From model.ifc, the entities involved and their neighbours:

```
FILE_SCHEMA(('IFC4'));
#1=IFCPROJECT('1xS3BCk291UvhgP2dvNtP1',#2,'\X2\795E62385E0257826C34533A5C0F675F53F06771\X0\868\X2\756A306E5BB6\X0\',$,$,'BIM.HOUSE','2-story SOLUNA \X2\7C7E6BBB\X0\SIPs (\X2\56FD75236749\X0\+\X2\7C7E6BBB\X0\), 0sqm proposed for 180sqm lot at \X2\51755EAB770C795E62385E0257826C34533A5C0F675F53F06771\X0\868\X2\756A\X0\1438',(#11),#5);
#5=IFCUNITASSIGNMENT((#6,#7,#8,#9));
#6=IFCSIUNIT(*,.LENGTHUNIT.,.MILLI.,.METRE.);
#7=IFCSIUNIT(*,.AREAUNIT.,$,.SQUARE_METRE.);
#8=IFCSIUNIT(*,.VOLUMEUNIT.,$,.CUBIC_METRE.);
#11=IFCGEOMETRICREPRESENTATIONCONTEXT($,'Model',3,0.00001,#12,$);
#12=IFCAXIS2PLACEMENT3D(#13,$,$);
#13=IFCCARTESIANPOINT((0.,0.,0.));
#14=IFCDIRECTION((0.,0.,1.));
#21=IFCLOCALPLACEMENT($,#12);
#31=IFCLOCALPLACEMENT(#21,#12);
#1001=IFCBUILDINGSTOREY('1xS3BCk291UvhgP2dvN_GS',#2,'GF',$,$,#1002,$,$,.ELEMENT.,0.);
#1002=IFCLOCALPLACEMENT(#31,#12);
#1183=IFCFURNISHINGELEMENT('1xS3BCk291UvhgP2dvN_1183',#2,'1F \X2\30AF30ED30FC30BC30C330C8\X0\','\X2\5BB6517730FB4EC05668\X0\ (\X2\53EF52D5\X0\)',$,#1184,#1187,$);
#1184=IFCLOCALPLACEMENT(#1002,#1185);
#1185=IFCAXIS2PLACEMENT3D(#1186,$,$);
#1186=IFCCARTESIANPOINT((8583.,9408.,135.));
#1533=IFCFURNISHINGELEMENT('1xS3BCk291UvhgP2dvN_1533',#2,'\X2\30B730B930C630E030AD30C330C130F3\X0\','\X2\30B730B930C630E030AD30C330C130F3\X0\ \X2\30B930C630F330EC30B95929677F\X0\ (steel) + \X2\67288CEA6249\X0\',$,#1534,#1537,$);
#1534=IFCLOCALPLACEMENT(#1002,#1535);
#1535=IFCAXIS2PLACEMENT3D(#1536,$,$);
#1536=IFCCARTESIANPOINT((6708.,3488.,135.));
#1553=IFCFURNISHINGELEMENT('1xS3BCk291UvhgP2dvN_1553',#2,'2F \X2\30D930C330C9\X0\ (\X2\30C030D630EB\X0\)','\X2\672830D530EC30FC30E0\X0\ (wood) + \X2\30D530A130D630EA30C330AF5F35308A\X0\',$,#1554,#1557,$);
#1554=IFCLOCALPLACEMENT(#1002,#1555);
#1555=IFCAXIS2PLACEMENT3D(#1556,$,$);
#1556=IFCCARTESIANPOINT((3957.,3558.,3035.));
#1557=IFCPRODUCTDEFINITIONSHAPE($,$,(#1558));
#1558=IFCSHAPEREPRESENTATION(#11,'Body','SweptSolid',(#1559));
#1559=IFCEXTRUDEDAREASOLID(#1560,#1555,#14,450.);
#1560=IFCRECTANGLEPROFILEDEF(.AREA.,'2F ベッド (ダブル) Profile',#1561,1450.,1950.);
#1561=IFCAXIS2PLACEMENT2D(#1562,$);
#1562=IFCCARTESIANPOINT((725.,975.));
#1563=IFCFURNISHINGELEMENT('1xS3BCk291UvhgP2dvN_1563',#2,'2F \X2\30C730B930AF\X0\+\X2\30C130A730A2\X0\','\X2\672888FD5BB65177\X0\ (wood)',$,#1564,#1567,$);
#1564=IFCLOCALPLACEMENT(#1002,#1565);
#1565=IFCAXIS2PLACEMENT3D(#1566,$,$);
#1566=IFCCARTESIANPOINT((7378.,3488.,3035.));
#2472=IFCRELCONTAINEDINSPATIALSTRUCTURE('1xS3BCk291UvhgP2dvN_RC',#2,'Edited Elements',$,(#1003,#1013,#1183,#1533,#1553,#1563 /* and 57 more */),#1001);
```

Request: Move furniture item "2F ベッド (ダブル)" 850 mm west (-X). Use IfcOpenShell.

```python
import ifcopenshell
import ifcopenshell.api.geometry
import ifcopenshell.util.placement
import ifcopenshell.util.unit

model = ifcopenshell.open("model.ifc")
unit_scale = ifcopenshell.util.unit.calculate_unit_scale(model)

item = model.by_guid("1xS3BCk291UvhgP2dvN_1553")
matrix = ifcopenshell.util.placement.get_local_placement(item.ObjectPlacement)
matrix[0, 3] -= 0.85 / unit_scale
ifcopenshell.api.geometry.edit_object_placement(model, product=item, matrix=matrix, is_si=False)

print(ifcopenshell.util.placement.get_local_placement(item.ObjectPlacement).round(3) + 0.0)

model.write("model_v2.ifc")
```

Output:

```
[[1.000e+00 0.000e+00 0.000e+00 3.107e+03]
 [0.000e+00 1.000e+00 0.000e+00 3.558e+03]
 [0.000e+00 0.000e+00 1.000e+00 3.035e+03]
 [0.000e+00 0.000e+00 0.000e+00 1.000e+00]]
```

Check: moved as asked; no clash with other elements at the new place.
